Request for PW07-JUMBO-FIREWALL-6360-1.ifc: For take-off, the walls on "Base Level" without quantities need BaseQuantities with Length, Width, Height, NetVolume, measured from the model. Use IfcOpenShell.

First a look at what the model holds.

```python
import ifcopenshell
import ifcopenshell.util.element
import ifcopenshell.util.unit

model = ifcopenshell.open("PW07-JUMBO-FIREWALL-6360-1.ifc")
print(model.schema)
for unit_type in ("LENGTHUNIT", "AREAUNIT", "VOLUMEUNIT"):
    print(unit_type, ifcopenshell.util.unit.calculate_unit_scale(model, unit_type))
storey = next(s for s in model.by_type("IfcBuildingStorey") if s.Name == "Base Level")
walls = [e for e in ifcopenshell.util.element.get_decomposition(storey) if e.is_a("IfcWall")]
for e in sorted(walls, key=lambda e: e.id()):
    print(e.id(), e.is_a(), e.Name, list(ifcopenshell.util.element.get_psets(e, qtos_only=True)), sep=" | ")
```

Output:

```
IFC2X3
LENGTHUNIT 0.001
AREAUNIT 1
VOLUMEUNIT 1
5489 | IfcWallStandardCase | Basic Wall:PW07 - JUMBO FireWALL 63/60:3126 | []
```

```python
import ifcopenshell
import ifcopenshell.api.pset
import ifcopenshell.geom
import ifcopenshell.util.element
import ifcopenshell.util.shape
import ifcopenshell.util.unit

model = ifcopenshell.open("PW07-JUMBO-FIREWALL-6360-1.ifc")
unit_scale = ifcopenshell.util.unit.calculate_unit_scale(model)
volume_scale = ifcopenshell.util.unit.calculate_unit_scale(model, "VOLUMEUNIT")
settings = ifcopenshell.geom.settings()

storey = next(s for s in model.by_type("IfcBuildingStorey") if s.Name == "Base Level")
walls = [e for e in ifcopenshell.util.element.get_decomposition(storey) if e.is_a("IfcWall")]

for e in sorted(walls, key=lambda e: e.id()):
    if ifcopenshell.util.element.get_psets(e, qtos_only=True, should_inherit=False):
        continue
    # Geometry comes back in metres, in the element's own axes.
    shape = ifcopenshell.geom.create_shape(settings, e)
    values = {
        "Length": ifcopenshell.util.shape.get_x(shape.geometry) / unit_scale,
        "Width": ifcopenshell.util.shape.get_y(shape.geometry) / unit_scale,
        "Height": ifcopenshell.util.shape.get_z(shape.geometry) / unit_scale,
        "NetVolume": ifcopenshell.util.shape.get_volume(shape.geometry) / volume_scale,
    }
    qto = ifcopenshell.api.pset.add_qto(model, product=e, name="BaseQuantities")
    ifcopenshell.api.pset.edit_qto(model, qto=qto, properties=values)
    print(e.id(), {k: round(v, 3) for k, v in values.items()})

model.write("PW07-JUMBO-FIREWALL-6360-1-out.ifc")
```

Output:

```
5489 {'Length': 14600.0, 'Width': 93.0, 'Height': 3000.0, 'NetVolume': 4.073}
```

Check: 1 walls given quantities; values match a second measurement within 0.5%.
